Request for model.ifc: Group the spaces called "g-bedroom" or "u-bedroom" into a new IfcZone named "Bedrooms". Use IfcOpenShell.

First a look at what the model holds.

```python
import ifcopenshell

model = ifcopenshell.open("model.ifc")
print(model.schema)
seen = {}
for space in model.by_type("IfcSpace"):
    seen[space.LongName] = seen.get(space.LongName, 0) + 1
for name, count in sorted(seen.items(), key=str):
    print(count, "x", name)
print("zones:", [z.Name for z in model.by_type("IfcZone")][:20])
```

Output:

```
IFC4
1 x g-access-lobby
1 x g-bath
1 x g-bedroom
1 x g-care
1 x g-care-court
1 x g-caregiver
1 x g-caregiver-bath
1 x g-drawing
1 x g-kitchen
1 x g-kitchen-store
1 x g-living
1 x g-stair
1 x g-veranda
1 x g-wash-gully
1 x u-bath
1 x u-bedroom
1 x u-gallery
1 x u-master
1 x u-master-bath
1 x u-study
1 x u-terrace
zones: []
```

```python
import ifcopenshell
import ifcopenshell.api.group
import ifcopenshell.api.root

model = ifcopenshell.open("model.ifc")

names = {"g-bedroom", "u-bedroom"}
spaces = [s for s in model.by_type("IfcSpace") if s.LongName in names]

zone = ifcopenshell.api.root.create_entity(model, ifc_class="IfcZone", name="Bedrooms")
ifcopenshell.api.group.assign_group(model, products=spaces, group=zone)
print(len(spaces), "spaces in", zone.Name)

model.write("model_edited.ifc")
```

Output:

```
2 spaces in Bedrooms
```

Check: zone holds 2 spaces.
